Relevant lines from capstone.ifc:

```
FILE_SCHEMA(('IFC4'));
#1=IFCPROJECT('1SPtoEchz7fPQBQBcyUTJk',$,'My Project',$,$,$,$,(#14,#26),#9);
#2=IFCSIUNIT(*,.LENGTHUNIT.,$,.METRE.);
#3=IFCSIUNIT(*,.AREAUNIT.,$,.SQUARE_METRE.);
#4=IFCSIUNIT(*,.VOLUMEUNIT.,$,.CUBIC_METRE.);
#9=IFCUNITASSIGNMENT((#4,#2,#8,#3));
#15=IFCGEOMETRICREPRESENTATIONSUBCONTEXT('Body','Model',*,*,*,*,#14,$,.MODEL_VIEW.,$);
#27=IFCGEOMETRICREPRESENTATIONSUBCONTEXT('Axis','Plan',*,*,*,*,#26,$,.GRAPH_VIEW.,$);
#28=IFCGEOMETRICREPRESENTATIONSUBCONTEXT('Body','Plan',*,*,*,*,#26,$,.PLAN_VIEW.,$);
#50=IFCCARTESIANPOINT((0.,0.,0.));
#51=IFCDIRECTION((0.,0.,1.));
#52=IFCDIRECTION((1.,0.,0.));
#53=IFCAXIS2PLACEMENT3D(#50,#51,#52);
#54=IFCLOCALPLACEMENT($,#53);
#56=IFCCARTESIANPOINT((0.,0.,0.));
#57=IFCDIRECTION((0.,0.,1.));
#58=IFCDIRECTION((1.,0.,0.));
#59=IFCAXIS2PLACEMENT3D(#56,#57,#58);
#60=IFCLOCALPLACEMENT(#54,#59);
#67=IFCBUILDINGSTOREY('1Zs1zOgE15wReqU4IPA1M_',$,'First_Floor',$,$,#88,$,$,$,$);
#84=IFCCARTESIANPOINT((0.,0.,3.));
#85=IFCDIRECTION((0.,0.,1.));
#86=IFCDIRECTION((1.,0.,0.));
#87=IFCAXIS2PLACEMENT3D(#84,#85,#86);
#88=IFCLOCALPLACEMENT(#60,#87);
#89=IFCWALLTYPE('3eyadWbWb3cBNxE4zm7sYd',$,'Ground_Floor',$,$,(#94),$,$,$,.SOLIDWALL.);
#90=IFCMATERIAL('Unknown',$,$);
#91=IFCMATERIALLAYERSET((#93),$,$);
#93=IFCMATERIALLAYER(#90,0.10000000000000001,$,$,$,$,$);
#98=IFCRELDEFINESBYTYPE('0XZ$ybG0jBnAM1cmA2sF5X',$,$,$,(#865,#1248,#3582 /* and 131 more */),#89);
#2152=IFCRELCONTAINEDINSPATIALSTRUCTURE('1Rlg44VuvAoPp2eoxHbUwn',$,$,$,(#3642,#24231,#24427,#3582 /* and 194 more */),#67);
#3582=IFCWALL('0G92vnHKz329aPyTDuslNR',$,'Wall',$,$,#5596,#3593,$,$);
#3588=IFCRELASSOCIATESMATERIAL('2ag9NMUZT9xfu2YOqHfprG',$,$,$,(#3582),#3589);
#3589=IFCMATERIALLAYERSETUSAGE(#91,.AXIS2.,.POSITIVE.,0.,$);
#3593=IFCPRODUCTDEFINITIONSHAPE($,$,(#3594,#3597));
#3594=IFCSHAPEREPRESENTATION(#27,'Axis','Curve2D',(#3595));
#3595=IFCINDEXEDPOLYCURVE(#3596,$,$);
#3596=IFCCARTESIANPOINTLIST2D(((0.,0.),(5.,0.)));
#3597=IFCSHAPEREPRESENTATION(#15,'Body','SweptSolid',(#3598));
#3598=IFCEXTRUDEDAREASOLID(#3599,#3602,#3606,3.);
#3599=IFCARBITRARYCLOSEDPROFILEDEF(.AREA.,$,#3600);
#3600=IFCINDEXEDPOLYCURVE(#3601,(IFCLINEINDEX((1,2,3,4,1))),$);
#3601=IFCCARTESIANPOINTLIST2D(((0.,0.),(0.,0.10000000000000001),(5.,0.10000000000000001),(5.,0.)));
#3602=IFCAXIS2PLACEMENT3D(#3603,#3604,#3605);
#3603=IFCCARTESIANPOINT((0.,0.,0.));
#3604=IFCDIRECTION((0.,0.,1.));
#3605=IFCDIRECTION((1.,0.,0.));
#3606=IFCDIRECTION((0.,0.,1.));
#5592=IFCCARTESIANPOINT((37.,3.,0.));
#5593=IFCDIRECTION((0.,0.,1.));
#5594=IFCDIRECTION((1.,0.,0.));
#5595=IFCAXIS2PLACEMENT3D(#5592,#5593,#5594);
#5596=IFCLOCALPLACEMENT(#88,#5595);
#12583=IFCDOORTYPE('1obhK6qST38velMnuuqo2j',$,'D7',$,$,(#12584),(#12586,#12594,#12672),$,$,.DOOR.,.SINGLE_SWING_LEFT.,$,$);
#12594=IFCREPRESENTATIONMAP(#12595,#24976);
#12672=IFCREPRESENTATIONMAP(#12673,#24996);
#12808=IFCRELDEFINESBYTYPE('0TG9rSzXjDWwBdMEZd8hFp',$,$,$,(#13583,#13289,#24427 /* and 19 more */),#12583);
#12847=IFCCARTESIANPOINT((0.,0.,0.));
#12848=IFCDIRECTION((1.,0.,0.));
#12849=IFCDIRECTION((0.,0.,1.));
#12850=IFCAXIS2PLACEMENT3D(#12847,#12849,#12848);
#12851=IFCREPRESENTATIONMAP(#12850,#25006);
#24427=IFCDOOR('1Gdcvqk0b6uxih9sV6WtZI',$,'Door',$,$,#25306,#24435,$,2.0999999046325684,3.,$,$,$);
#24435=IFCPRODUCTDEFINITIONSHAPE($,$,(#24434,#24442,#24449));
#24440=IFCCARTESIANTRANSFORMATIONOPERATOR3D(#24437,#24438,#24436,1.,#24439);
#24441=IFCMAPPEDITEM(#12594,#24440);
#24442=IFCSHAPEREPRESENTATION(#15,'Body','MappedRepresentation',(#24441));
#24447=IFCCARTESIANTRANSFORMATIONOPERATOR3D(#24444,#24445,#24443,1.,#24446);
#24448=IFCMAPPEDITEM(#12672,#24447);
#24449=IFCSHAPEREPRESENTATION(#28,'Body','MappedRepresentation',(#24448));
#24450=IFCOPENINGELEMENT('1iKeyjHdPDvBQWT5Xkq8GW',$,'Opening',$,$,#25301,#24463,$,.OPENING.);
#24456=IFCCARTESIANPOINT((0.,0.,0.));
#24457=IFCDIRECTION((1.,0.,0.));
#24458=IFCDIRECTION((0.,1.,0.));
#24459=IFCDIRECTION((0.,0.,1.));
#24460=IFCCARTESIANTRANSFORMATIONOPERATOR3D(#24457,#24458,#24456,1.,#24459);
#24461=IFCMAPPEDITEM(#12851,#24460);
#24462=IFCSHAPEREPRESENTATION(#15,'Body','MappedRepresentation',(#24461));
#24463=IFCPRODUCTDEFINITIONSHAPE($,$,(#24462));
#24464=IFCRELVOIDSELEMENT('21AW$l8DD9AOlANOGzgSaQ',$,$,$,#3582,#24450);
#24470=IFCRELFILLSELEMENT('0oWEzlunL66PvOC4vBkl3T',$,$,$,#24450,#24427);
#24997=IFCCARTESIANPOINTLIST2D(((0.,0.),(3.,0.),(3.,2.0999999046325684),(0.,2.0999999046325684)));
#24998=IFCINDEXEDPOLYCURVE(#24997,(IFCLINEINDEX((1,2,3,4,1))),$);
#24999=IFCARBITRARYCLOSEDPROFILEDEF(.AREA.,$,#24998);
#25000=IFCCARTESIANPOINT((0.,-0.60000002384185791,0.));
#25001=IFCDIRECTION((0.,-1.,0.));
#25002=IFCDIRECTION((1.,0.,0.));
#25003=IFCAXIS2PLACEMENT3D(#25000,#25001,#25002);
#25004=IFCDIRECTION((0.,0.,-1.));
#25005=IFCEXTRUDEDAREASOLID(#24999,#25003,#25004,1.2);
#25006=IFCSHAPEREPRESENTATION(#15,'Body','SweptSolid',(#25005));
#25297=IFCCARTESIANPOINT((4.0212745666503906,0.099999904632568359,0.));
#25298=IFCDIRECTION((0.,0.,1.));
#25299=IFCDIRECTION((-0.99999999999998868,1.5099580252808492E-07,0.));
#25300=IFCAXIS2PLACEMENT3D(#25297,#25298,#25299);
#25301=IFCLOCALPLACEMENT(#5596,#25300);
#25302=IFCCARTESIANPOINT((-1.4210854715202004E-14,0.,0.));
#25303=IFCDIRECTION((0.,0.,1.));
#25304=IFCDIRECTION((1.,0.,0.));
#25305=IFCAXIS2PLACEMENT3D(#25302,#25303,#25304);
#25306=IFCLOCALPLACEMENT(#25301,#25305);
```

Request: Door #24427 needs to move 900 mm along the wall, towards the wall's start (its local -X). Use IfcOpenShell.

```python
import ifcopenshell
import ifcopenshell.api.geometry
import ifcopenshell.util.placement

model = ifcopenshell.open("capstone.ifc")

door = model.by_guid("1Gdcvqk0b6uxih9sV6WtZI")
opening = door.FillsVoids[0].RelatingOpeningElement
wall = opening.VoidsElements[0].RelatingBuildingElement

wall_matrix = ifcopenshell.util.placement.get_local_placement(wall.ObjectPlacement)
shift = wall_matrix[:3, 0] * -0.9
before = ifcopenshell.util.placement.get_local_placement(door.ObjectPlacement)[:3, 3].copy()

# The door is placed relative to its opening, so it follows when the opening moves.
matrix = ifcopenshell.util.placement.get_local_placement(opening.ObjectPlacement)
matrix[:3, 3] += shift
ifcopenshell.api.geometry.edit_object_placement(
    model, product=opening, matrix=matrix, is_si=False, should_transform_children=True
)

after = ifcopenshell.util.placement.get_local_placement(door.ObjectPlacement)[:3, 3]
print("door moved by", (after - before).round(3) + 0.0)

model.write("capstone_edited.ifc")
```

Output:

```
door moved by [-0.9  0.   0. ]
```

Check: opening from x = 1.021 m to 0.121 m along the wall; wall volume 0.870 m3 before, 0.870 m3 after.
